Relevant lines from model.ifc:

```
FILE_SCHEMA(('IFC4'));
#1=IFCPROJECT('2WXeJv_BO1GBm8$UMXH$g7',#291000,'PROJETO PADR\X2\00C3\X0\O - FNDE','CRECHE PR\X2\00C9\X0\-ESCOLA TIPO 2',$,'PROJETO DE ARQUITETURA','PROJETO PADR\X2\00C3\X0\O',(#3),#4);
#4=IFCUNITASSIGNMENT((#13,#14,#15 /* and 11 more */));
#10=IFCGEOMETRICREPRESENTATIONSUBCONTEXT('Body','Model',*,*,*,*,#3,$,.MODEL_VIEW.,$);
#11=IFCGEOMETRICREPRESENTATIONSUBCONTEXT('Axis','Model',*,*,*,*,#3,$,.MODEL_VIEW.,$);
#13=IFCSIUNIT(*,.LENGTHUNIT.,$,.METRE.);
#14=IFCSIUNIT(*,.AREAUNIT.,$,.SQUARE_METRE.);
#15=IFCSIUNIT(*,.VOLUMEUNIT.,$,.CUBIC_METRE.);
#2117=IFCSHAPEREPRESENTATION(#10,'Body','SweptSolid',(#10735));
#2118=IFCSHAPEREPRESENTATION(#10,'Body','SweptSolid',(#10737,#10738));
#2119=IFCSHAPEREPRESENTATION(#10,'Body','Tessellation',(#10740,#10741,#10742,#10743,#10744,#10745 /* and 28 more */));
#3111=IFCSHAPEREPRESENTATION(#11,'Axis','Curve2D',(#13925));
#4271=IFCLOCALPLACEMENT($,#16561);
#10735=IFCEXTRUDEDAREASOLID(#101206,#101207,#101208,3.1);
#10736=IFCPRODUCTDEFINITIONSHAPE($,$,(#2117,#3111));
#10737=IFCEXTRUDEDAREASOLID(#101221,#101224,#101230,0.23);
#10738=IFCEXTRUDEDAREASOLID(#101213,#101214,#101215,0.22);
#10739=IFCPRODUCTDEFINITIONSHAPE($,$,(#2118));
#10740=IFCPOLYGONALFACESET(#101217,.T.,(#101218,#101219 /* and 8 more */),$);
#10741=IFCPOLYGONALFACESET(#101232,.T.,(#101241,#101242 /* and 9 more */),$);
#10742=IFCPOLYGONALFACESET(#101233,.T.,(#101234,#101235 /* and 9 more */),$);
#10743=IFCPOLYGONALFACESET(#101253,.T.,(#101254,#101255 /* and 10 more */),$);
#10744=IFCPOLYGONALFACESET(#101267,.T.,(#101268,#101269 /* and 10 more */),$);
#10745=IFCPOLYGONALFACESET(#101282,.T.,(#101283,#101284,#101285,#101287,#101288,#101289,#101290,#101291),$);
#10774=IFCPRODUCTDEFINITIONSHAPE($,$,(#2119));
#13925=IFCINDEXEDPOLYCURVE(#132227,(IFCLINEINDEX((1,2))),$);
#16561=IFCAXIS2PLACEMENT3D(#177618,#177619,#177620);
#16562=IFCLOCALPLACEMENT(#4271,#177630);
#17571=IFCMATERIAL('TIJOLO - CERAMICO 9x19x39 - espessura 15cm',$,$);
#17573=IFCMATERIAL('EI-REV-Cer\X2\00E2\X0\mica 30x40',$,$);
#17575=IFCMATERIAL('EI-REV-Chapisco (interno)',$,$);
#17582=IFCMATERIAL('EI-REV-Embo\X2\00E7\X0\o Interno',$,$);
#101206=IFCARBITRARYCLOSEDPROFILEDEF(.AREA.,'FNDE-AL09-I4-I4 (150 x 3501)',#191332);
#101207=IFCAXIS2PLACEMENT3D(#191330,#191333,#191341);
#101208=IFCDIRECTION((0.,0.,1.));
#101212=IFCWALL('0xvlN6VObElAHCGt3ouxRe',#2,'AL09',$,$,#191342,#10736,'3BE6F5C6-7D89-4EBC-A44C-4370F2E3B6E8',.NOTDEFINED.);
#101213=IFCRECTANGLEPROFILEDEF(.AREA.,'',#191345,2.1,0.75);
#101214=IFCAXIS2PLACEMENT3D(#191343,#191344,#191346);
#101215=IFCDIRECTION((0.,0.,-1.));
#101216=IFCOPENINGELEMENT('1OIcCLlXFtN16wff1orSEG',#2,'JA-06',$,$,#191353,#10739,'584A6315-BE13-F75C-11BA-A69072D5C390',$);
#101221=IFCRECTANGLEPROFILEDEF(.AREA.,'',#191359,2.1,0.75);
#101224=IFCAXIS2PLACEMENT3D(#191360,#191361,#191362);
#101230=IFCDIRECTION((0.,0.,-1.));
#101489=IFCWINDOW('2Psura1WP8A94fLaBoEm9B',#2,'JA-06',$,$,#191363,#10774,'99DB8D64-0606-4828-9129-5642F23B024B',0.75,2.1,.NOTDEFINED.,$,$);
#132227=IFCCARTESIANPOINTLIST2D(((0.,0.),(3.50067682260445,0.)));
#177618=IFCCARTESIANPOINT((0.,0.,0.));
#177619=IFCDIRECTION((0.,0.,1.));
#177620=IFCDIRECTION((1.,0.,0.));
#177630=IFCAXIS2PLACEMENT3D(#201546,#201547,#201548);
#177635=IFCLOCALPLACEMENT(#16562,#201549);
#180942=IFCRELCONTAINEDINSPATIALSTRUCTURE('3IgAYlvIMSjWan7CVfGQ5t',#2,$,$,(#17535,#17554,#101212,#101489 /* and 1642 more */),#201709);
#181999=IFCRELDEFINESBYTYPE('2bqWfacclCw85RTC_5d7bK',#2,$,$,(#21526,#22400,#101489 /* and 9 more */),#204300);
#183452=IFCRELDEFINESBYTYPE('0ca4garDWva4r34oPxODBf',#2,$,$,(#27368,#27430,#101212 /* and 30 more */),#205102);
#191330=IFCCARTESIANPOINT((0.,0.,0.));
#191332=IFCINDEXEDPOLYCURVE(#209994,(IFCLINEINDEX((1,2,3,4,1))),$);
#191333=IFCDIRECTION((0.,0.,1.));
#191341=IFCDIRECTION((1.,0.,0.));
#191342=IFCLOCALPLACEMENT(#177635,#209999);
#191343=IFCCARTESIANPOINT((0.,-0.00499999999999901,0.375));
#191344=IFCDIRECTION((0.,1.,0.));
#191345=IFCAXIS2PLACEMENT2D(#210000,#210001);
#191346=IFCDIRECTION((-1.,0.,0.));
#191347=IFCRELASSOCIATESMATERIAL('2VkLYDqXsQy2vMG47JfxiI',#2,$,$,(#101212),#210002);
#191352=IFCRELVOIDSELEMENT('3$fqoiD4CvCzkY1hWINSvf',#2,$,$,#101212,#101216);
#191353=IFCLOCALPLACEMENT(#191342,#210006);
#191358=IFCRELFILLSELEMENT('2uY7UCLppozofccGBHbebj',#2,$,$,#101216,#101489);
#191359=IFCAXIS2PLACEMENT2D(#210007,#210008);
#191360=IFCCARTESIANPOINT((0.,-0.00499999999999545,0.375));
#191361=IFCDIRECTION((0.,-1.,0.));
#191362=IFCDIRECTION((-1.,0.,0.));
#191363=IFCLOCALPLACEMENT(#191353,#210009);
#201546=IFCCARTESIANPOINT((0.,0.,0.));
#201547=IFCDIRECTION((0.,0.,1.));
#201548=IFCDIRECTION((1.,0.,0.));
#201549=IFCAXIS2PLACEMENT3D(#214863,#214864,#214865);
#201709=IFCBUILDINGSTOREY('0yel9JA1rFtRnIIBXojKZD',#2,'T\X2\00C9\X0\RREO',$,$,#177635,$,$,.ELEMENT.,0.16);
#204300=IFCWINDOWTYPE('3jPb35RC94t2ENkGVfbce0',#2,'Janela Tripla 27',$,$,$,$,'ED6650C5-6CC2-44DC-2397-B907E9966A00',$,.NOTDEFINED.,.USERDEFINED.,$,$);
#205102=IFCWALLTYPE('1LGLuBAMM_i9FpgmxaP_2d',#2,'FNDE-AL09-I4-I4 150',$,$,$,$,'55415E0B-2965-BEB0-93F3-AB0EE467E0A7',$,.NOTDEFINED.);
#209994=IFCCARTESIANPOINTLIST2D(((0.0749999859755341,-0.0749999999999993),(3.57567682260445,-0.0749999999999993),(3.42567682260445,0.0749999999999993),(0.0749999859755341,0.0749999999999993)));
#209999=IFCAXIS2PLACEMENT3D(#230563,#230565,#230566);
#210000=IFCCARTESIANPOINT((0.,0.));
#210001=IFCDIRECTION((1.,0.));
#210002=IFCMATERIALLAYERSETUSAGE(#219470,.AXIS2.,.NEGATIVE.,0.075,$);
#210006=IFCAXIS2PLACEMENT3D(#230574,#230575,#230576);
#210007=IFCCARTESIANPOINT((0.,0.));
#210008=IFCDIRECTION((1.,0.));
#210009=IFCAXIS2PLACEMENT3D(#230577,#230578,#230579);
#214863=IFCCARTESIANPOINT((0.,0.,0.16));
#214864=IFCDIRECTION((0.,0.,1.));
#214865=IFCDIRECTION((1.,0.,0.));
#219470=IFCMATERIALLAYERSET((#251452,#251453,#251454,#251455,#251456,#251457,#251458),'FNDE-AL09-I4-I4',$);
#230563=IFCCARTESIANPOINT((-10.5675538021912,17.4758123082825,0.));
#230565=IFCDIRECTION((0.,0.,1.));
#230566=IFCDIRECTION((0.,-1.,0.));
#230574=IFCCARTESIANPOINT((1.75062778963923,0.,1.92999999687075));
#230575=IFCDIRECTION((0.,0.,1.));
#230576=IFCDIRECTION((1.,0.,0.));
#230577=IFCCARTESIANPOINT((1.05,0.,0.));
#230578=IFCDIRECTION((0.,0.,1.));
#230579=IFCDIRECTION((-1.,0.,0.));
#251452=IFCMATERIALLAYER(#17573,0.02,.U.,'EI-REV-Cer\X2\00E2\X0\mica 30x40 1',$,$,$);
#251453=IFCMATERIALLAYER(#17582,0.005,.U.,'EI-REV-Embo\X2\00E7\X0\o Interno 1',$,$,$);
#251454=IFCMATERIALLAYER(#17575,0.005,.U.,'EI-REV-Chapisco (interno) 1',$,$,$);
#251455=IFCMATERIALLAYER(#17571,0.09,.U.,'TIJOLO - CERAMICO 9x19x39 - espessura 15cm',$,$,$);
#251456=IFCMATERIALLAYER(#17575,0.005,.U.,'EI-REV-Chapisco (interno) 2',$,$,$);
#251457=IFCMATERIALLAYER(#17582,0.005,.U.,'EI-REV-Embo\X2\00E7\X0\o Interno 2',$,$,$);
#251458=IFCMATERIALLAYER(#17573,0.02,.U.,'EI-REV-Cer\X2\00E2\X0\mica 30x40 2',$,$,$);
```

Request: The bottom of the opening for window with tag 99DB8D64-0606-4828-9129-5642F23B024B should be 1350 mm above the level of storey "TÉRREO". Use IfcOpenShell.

```python
import numpy as np
import ifcopenshell
import ifcopenshell.api.geometry
import ifcopenshell.geom
import ifcopenshell.util.element
import ifcopenshell.util.placement
import ifcopenshell.util.shape
import ifcopenshell.util.unit

model = ifcopenshell.open("model.ifc")
unit_scale = ifcopenshell.util.unit.calculate_unit_scale(model)

window = model.by_id(101489)
opening = window.FillsVoids[0].RelatingOpeningElement
storey = ifcopenshell.util.element.get_container(window, ifc_class="IfcBuildingStorey")
level = ifcopenshell.util.placement.get_local_placement(storey.ObjectPlacement)[2, 3]

# The opening's origin need not be at the sill, so measure its lowest point.
shape = ifcopenshell.geom.create_shape(ifcopenshell.geom.settings(), opening)
bottom = ifcopenshell.util.shape.get_shape_bottom_elevation(shape, shape.geometry) / unit_scale
dz = level + 1.35 - bottom

shift = np.array([0.0, 0.0, dz])
# The window is placed relative to its opening, so it follows when the opening moves.
matrix = ifcopenshell.util.placement.get_local_placement(opening.ObjectPlacement)
matrix[:3, 3] += shift
ifcopenshell.api.geometry.edit_object_placement(
    model, product=opening, matrix=matrix, is_si=False, should_transform_children=True
)

print(f"moved by {dz * unit_scale:+.3f} m")

model.write("model_edited.ifc")
```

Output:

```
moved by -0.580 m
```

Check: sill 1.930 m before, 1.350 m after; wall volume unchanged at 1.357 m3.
